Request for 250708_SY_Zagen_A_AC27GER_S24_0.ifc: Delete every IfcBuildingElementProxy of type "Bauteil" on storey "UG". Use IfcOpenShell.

First a look at what the model holds.

```python
import ifcopenshell
import ifcopenshell.util.element

model = ifcopenshell.open("250708_SY_Zagen_A_AC27GER_S24_0.ifc")
print(model.schema)
storey = next(s for s in model.by_type("IfcBuildingStorey") if s.Name == "UG")
proxies = [e for e in ifcopenshell.util.element.get_decomposition(storey) if e.is_a("IfcBuildingElementProxy")]
seen = {}
for e in proxies:
    element_type = ifcopenshell.util.element.get_type(e)
    name = element_type.Name if element_type not in (None, e) else None
    seen[name] = seen.get(name, 0) + 1
for name, count in sorted(seen.items(), key=str):
    print(count, "x", name)
```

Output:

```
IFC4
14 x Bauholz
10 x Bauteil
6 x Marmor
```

```python
import ifcopenshell
import ifcopenshell.api.root
import ifcopenshell.util.element

model = ifcopenshell.open("250708_SY_Zagen_A_AC27GER_S24_0.ifc")

storey = next(s for s in model.by_type("IfcBuildingStorey") if s.Name == "UG")
proxies = [e for e in ifcopenshell.util.element.get_decomposition(storey) if e.is_a("IfcBuildingElementProxy")]
targets = [e for e in proxies if (t := ifcopenshell.util.element.get_type(e)) not in (None, e) and t.Name == "Bauteil"]

for e in targets:
    ifcopenshell.api.root.remove_product(model, product=e)
print(len(targets), "removed")

model.write("250708_SY_Zagen_A_AC27GER_S24_0-out.ifc")
```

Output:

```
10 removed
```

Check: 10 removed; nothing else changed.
